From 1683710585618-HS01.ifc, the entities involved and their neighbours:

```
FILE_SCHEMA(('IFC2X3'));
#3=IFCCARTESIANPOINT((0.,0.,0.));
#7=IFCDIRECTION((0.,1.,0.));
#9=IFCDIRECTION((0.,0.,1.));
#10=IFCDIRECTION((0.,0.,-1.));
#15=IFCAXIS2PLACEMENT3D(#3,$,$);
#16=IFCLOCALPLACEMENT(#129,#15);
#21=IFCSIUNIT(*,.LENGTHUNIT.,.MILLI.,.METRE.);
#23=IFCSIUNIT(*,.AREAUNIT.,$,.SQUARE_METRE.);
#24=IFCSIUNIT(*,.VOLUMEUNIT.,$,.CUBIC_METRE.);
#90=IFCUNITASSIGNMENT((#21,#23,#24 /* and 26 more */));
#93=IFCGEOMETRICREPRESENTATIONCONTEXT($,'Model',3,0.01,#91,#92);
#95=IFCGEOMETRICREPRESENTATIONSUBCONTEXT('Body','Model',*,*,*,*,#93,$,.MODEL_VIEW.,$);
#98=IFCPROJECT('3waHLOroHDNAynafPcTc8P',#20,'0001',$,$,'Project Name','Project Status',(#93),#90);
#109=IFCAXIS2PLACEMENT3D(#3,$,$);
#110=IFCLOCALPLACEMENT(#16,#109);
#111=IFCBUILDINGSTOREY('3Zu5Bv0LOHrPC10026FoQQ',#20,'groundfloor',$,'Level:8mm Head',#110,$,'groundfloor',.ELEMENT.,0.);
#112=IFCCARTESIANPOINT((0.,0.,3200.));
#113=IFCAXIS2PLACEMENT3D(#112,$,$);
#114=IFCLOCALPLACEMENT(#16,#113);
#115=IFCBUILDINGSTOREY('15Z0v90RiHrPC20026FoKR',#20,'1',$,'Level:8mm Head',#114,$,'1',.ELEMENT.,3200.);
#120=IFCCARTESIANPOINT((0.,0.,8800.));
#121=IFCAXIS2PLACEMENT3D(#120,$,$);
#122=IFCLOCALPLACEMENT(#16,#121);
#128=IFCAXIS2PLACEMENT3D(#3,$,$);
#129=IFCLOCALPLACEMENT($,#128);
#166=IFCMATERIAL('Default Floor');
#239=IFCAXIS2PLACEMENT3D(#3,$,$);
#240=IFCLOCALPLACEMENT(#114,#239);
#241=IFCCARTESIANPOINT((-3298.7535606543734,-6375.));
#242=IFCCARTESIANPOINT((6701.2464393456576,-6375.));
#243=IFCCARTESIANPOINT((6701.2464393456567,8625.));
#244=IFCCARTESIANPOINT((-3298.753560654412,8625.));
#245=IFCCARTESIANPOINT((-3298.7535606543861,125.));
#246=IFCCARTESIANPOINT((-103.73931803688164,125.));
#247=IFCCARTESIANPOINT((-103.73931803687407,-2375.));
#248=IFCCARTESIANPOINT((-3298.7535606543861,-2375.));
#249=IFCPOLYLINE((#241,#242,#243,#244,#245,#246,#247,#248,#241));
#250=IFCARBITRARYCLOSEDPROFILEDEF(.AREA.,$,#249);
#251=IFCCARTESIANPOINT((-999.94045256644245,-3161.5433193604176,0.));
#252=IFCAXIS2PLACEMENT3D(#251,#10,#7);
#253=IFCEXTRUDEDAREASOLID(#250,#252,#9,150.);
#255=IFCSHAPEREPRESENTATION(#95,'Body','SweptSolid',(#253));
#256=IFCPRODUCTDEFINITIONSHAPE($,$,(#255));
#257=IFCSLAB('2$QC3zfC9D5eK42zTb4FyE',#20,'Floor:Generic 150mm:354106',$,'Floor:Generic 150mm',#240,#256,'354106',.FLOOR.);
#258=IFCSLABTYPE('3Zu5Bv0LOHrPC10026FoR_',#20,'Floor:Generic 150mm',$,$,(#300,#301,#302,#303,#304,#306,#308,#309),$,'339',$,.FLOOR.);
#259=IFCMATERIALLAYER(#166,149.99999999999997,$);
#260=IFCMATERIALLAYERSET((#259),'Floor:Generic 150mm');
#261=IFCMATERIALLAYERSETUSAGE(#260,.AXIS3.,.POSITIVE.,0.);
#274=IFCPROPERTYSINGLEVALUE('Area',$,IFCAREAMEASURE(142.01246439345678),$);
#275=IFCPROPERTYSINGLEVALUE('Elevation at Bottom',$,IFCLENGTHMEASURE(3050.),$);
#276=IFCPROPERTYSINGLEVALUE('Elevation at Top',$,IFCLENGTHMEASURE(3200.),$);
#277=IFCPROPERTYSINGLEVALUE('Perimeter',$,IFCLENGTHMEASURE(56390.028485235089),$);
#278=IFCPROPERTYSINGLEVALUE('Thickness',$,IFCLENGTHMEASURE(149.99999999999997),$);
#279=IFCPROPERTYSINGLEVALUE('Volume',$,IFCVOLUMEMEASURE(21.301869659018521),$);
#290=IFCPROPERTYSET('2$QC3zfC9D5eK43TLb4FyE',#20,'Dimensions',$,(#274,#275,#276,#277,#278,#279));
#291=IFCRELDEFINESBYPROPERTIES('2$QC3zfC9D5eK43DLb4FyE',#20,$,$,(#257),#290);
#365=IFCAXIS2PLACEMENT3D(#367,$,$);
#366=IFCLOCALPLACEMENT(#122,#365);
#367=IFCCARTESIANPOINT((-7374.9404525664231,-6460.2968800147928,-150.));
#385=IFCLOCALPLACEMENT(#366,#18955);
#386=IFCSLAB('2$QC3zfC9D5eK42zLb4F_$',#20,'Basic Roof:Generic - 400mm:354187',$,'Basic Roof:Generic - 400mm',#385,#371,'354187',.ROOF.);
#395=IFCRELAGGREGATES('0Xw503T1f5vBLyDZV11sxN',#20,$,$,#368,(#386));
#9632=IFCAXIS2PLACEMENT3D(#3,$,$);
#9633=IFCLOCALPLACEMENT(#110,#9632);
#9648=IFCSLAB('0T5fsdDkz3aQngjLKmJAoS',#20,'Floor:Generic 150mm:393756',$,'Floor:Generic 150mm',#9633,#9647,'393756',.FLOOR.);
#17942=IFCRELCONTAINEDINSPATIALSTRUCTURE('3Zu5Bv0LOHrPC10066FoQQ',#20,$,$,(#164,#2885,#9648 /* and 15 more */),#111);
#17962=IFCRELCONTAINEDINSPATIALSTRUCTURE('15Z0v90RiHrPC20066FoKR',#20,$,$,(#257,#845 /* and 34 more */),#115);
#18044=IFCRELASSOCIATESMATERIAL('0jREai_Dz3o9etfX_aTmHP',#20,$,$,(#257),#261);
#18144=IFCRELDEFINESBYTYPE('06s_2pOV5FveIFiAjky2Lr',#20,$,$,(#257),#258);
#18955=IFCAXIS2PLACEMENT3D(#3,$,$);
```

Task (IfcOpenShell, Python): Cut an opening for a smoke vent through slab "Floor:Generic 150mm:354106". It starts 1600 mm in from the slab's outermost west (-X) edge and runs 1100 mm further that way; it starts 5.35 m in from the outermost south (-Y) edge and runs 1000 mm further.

```python
import numpy as np
import ifcopenshell
import ifcopenshell.api.feature
import ifcopenshell.api.geometry
import ifcopenshell.api.pset
import ifcopenshell.api.root
import ifcopenshell.geom
import ifcopenshell.util.element
import ifcopenshell.util.placement
import ifcopenshell.util.representation
import ifcopenshell.util.shape
import ifcopenshell.util.unit

model = ifcopenshell.open("1683710585618-HS01.ifc")
unit_scale = ifcopenshell.util.unit.calculate_unit_scale(model)
area_scale = ifcopenshell.util.unit.calculate_unit_scale(model, "AREAUNIT")
volume_scale = ifcopenshell.util.unit.calculate_unit_scale(model, "VOLUMEUNIT")
settings = ifcopenshell.geom.settings()


def volume(element):
    """Net volume in cubic metres, openings subtracted."""
    shape = ifcopenshell.geom.create_shape(settings, element)
    return ifcopenshell.util.shape.get_volume(shape.geometry)


slab = model.by_id(257)
before = volume(slab)

# Extent in the slab's own axes, in metres. The edges named are its -X and -Y sides.
slab_shape = ifcopenshell.geom.create_shape(settings, slab)
vertices = ifcopenshell.util.shape.get_vertices(slab_shape.geometry)
x_min, y_min, bottom = vertices.min(axis=0)
top = vertices[:, 2].max()

opening = ifcopenshell.api.root.create_entity(model, ifc_class="IfcOpeningElement", name="Smoke vent opening")
context = ifcopenshell.util.representation.get_context(model, "Model", "Body", "MODEL_VIEW")
width, depth = 1.1, 1
outline = [(0.0, 0.0), (width, 0.0), (width, depth), (0.0, depth), (0.0, 0.0)]
# Overshoot both faces by 50 mm so the cut is clean.
shape = ifcopenshell.api.geometry.add_slab_representation(
    model, context=context, depth=top - bottom + 0.1, polyline=outline
)
ifcopenshell.api.geometry.assign_representation(model, product=opening, representation=shape)

matrix = ifcopenshell.util.placement.get_local_placement(slab.ObjectPlacement)
matrix[:, 3] = matrix @ np.append(np.array([x_min + 1.6, y_min + 5.35, bottom - 0.05]) / unit_scale, 1.0)
ifcopenshell.api.geometry.edit_object_placement(model, product=opening, matrix=matrix, is_si=False)
ifcopenshell.api.feature.add_feature(model, feature=opening, element=slab)

after = volume(slab)

# Update the slab's stored quantities.
pset = model.by_id(ifcopenshell.util.element.get_pset(slab, "Dimensions", should_inherit=False)["id"])
ifcopenshell.api.pset.edit_pset(model, pset=pset, properties={
    "Area": model.create_entity("IfcAreaMeasure", after / (top - bottom) / area_scale),
    "Volume": model.create_entity("IfcVolumeMeasure", after / volume_scale),
})

print(f"slab volume {before:.3f} -> {after:.3f} m3")

model.write("1683710585618-HS01-out.ifc")
```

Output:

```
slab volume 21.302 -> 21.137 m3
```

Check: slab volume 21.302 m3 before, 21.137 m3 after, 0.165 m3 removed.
